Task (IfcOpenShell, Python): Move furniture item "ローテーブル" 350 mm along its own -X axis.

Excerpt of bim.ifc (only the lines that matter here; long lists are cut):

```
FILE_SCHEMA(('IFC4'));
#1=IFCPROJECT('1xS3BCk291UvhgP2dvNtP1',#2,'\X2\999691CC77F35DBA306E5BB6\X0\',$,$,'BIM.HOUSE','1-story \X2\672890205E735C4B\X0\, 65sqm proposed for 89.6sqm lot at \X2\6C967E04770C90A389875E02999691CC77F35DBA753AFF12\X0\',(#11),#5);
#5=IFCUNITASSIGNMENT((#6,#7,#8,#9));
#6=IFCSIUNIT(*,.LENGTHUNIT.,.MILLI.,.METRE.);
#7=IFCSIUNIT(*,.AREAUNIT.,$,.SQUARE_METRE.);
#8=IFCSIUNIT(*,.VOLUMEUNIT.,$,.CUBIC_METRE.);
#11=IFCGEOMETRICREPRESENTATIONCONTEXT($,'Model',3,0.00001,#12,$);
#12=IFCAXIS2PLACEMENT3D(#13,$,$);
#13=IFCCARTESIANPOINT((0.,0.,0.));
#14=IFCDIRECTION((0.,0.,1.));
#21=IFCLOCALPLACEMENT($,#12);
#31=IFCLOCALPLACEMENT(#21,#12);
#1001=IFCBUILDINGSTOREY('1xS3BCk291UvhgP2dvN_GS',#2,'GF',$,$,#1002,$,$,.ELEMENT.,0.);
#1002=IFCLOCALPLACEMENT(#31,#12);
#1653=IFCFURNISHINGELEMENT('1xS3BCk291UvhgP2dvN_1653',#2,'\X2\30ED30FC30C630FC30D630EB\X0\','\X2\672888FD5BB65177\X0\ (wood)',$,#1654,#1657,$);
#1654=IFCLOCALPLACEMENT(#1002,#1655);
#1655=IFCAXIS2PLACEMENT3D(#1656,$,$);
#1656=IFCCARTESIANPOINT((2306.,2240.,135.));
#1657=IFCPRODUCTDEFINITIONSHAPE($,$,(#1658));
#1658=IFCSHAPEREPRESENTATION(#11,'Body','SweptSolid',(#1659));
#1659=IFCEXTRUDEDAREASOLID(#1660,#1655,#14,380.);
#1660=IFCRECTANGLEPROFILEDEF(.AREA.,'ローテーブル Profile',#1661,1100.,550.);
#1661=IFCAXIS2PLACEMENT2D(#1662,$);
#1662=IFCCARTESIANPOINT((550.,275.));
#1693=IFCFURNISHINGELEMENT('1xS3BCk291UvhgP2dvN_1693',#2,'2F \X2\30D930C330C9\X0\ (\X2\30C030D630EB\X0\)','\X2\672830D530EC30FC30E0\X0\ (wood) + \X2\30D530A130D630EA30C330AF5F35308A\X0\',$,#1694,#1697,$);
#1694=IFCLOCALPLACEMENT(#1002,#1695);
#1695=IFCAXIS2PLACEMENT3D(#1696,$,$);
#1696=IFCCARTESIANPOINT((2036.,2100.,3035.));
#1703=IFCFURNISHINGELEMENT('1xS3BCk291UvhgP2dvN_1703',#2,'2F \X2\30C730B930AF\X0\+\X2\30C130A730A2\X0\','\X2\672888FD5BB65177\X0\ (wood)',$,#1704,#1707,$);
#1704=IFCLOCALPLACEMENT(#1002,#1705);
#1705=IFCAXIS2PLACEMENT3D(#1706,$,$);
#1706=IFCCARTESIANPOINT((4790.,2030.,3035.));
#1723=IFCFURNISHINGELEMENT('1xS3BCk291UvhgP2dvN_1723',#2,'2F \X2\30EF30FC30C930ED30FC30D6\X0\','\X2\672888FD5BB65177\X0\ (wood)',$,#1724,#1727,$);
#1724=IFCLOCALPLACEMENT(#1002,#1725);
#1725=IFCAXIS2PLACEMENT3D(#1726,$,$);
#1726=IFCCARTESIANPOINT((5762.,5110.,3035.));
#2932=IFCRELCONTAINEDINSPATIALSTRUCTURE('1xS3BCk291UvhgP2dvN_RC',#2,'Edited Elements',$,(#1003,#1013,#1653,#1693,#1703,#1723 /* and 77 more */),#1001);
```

```python
import ifcopenshell
import ifcopenshell.api.geometry
import ifcopenshell.util.placement
import ifcopenshell.util.unit

model = ifcopenshell.open("bim.ifc")
unit_scale = ifcopenshell.util.unit.calculate_unit_scale(model)

item = model.by_guid("1xS3BCk291UvhgP2dvN_1653")
matrix = ifcopenshell.util.placement.get_local_placement(item.ObjectPlacement)
matrix[:3, 3] -= matrix[:3, 0] * 0.35 / unit_scale
ifcopenshell.api.geometry.edit_object_placement(model, product=item, matrix=matrix, is_si=False)

print(ifcopenshell.util.placement.get_local_placement(item.ObjectPlacement).round(3) + 0.0)

model.write("bim_updated.ifc")
```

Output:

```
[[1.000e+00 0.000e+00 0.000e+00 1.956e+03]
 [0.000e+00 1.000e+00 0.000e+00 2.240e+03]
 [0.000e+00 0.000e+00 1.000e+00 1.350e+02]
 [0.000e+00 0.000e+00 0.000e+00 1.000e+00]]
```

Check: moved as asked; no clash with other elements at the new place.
